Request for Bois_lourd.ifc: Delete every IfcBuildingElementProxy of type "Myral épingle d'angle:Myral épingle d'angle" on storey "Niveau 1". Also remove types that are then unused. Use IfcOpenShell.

First a look at what the model holds.

```python
import ifcopenshell
import ifcopenshell.util.element

model = ifcopenshell.open("Bois_lourd.ifc")
print(model.schema)
storey = next(s for s in model.by_type("IfcBuildingStorey") if s.Name == "Niveau 1")
proxies = [e for e in ifcopenshell.util.element.get_decomposition(storey) if e.is_a("IfcBuildingElementProxy")]
seen = {}
for e in proxies:
    element_type = ifcopenshell.util.element.get_type(e)
    name = element_type.Name if element_type not in (None, e) else None
    seen[name] = seen.get(name, 0) + 1
for name, count in sorted(seen.items(), key=str):
    print(count, "x", name)
```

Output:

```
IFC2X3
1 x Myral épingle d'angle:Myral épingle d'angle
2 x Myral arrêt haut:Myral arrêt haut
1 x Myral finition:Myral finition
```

```python
import ifcopenshell
import ifcopenshell.api.root
import ifcopenshell.util.element

model = ifcopenshell.open("Bois_lourd.ifc")

storey = next(s for s in model.by_type("IfcBuildingStorey") if s.Name == "Niveau 1")
proxies = [e for e in ifcopenshell.util.element.get_decomposition(storey) if e.is_a("IfcBuildingElementProxy")]
targets = [e for e in proxies if (t := ifcopenshell.util.element.get_type(e)) not in (None, e) and t.Name == "Myral épingle d'angle:Myral épingle d'angle"]
types = {ifcopenshell.util.element.get_type(e) for e in targets} - {None, *targets}

for e in targets:
    ifcopenshell.api.root.remove_product(model, product=e)
print(len(targets), "removed")

unused = [t for t in types if not ifcopenshell.util.element.get_types(t)]
for t in unused:
    ifcopenshell.api.root.remove_product(model, product=t)
print(len(unused), "unused types removed")

model.write("Bois_lourd-out.ifc")
```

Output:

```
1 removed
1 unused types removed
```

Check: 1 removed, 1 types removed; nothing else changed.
